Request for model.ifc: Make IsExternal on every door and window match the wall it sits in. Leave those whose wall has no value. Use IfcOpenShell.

First a look at what the model holds.

```python
import ifcopenshell
import ifcopenshell.util.element

model = ifcopenshell.open("model.ifc")
print(model.schema)
seen = {}
for e in model.by_type("IfcDoor") + model.by_type("IfcWindow"):
    if not e.FillsVoids:
        continue
    host = e.FillsVoids[0].RelatingOpeningElement.VoidsElements[0].RelatingBuildingElement
    own = ifcopenshell.util.element.get_pset(e, f"Pset_{e.is_a()[3:].removesuffix('StandardCase')}Common", "IsExternal")
    wall = ifcopenshell.util.element.get_pset(host, "Pset_WallCommon", "IsExternal")
    seen[e.is_a(), own, wall] = seen.get((e.is_a(), own, wall), 0) + 1
for (cls, own, wall), count in sorted(seen.items(), key=str):
    print(count, cls, "IsExternal:", own, "| host wall:", wall)
```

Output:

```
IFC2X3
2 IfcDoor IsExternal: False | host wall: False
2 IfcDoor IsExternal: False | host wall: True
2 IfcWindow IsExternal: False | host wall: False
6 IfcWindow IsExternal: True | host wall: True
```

```python
import ifcopenshell
import ifcopenshell.api.pset
import ifcopenshell.util.element

model = ifcopenshell.open("model.ifc")

count = 0
for ifc_class, pset_name in (("IfcDoor", "Pset_DoorCommon"), ("IfcWindow", "Pset_WindowCommon")):
    for e in model.by_type(ifc_class):
        if not e.FillsVoids:
            continue
        host = e.FillsVoids[0].RelatingOpeningElement.VoidsElements[0].RelatingBuildingElement
        external = ifcopenshell.util.element.get_pset(host, "Pset_WallCommon", "IsExternal")
        if external is None or ifcopenshell.util.element.get_pset(e, pset_name, "IsExternal") == external:
            continue
        pset = ifcopenshell.api.pset.add_pset(model, product=e, name=pset_name)
        ifcopenshell.api.pset.edit_pset(model, pset=pset, properties={"IsExternal": external})
        count += 1

print(count, "updated")

model.write("model_edited.ifc")
```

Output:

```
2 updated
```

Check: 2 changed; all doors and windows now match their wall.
